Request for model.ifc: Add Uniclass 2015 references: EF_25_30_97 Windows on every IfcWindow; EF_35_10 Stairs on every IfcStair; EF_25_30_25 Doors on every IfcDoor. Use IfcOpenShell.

First a look at what the model holds.

```python
import ifcopenshell

model = ifcopenshell.open("model.ifc")
print(model.schema)
print("classifications:", [c.Name for c in model.by_type("IfcClassification")])
for ifc_class in ("IfcDoor", "IfcRoof", "IfcStair", "IfcWall", "IfcWindow"):
    print(ifc_class, len(model.by_type(ifc_class)))
```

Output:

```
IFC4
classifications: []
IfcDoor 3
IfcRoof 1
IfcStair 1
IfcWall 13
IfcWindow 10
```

```python
import ifcopenshell
import ifcopenshell.api.classification

model = ifcopenshell.open("model.ifc")

system = ifcopenshell.api.classification.add_classification(model, classification="Uniclass 2015")

codes = {
    "IfcWindow": ("EF_25_30_97", "Windows"),
    "IfcStair": ("EF_35_10", "Stairs"),
    "IfcDoor": ("EF_25_30_25", "Doors"),
}
for ifc_class, (code, name) in codes.items():
    products = model.by_type(ifc_class)
    ifcopenshell.api.classification.add_reference(
        model, products=products, classification=system, identification=code, name=name
    )
    print(code, len(products))

model.write("model_edited.ifc")
```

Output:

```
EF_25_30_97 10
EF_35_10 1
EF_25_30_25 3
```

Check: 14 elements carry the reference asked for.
